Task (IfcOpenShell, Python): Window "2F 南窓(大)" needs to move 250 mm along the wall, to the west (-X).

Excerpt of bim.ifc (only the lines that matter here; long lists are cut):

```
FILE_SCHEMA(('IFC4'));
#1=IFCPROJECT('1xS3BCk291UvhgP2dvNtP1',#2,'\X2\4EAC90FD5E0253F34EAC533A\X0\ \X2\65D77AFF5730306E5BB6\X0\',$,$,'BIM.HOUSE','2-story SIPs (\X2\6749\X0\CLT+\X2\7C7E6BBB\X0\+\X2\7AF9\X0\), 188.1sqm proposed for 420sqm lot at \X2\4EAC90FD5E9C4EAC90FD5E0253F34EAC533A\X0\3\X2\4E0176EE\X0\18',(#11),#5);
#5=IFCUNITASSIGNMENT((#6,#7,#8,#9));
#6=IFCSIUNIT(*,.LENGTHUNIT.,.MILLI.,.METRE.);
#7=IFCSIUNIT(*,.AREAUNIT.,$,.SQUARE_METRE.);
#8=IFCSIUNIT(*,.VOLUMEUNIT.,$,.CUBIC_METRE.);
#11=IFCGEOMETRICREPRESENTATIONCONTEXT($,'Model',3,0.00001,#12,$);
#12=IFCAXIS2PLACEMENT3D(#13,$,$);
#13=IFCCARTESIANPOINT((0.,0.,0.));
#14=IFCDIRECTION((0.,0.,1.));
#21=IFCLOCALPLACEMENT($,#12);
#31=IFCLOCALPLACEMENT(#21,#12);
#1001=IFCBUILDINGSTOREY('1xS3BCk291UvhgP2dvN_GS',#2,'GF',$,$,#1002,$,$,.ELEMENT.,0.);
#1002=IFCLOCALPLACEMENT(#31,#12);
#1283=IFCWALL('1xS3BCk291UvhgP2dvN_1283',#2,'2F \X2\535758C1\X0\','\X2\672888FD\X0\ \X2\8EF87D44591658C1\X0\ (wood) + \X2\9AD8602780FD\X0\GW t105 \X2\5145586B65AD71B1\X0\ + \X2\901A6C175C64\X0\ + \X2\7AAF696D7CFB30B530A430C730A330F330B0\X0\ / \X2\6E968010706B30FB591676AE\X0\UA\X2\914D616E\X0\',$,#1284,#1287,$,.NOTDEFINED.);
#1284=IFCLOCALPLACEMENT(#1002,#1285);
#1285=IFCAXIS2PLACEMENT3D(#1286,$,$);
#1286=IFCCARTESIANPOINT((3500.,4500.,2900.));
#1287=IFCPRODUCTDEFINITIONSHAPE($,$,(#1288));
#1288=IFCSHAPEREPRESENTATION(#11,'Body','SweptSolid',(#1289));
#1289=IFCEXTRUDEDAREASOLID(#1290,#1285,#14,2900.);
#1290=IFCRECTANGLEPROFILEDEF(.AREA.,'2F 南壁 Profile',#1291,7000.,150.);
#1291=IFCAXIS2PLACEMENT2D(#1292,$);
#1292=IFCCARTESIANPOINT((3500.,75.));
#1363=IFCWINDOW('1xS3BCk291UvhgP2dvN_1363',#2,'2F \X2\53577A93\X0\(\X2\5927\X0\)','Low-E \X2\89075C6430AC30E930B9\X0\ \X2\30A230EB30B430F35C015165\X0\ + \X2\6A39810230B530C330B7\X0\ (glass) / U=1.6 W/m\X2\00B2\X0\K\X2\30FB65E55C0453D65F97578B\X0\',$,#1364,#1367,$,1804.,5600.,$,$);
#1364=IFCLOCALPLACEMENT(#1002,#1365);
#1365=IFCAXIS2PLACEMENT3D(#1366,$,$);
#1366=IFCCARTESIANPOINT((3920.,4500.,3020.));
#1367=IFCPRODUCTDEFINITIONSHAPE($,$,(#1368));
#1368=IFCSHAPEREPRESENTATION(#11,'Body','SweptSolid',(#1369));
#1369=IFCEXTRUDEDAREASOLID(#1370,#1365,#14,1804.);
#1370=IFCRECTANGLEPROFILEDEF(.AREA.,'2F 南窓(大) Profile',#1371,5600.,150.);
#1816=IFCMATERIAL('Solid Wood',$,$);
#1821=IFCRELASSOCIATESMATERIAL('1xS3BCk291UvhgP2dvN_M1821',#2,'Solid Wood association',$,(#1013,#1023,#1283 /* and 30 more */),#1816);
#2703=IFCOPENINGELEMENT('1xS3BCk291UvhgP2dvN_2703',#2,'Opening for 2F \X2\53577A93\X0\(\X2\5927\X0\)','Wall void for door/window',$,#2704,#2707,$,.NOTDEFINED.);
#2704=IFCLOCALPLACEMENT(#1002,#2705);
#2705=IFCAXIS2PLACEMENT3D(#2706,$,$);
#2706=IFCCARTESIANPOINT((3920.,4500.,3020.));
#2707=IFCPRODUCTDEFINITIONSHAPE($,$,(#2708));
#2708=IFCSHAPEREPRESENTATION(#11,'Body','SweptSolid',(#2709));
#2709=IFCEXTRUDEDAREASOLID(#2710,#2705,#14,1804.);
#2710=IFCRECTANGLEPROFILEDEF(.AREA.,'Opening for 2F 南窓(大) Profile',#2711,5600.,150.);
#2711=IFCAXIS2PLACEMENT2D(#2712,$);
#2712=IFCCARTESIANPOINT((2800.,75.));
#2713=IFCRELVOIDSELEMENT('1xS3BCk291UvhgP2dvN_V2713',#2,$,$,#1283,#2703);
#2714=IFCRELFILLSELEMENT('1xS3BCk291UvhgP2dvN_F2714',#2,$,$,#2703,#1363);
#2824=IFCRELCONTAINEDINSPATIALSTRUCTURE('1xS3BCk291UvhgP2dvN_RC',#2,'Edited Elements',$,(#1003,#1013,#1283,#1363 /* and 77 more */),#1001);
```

```python
import ifcopenshell
import ifcopenshell.api.geometry
import ifcopenshell.util.placement
import ifcopenshell.util.unit

model = ifcopenshell.open("bim.ifc")
unit_scale = ifcopenshell.util.unit.calculate_unit_scale(model)

window = model.by_guid("1xS3BCk291UvhgP2dvN_1363")
opening = window.FillsVoids[0].RelatingOpeningElement
wall = opening.VoidsElements[0].RelatingBuildingElement

wall_matrix = ifcopenshell.util.placement.get_local_placement(wall.ObjectPlacement)
shift = wall_matrix[:3, 0] * -0.25 / unit_scale
before = ifcopenshell.util.placement.get_local_placement(window.ObjectPlacement)[:3, 3].copy()

# The window is not placed relative to its opening, so move both.
for product in (opening, window):
    matrix = ifcopenshell.util.placement.get_local_placement(product.ObjectPlacement)
    matrix[:3, 3] += shift
    ifcopenshell.api.geometry.edit_object_placement(model, product=product, matrix=matrix, is_si=False)

after = ifcopenshell.util.placement.get_local_placement(window.ObjectPlacement)[:3, 3]
print("window moved by", (after - before).round(3) + 0.0)

model.write("bim_rev.ifc")
```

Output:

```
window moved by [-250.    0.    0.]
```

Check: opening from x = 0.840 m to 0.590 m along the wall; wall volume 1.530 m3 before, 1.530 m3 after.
